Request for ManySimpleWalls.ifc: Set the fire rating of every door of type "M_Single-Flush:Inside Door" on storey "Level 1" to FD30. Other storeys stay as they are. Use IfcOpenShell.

First a look at what the model holds.

```python
import ifcopenshell
import ifcopenshell.util.element

model = ifcopenshell.open("ManySimpleWalls.ifc")
print(model.schema)
storey = next(s for s in model.by_type("IfcBuildingStorey") if s.Name == "Level 1")
doors = [e for e in ifcopenshell.util.element.get_decomposition(storey) if e.is_a("IfcDoor")]
seen = {}
for e in doors:
    element_type = ifcopenshell.util.element.get_type(e)
    key = (element_type.Name if element_type != e and element_type else None, ifcopenshell.util.element.get_pset(e, "Pset_DoorCommon", "FireRating"))
    seen[key] = seen.get(key, 0) + 1
for (name, value), count in sorted(seen.items(), key=str):
    print(count, "x", name, "|", value)
```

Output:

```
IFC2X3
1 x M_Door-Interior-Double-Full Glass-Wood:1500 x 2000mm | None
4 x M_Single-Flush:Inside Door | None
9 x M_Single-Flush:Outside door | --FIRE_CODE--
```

```python
import ifcopenshell
import ifcopenshell.api.pset
import ifcopenshell.util.element

model = ifcopenshell.open("ManySimpleWalls.ifc")

storey = next(s for s in model.by_type("IfcBuildingStorey") if s.Name == "Level 1")
doors = [e for e in ifcopenshell.util.element.get_decomposition(storey) if e.is_a("IfcDoor")]

count = 0
for e in doors:
    element_type = ifcopenshell.util.element.get_type(e)
    if element_type in (None, e) or element_type.Name != "M_Single-Flush:Inside Door":
        continue
    # add_pset returns the element's existing set when there is one.
    pset = ifcopenshell.api.pset.add_pset(model, product=e, name="Pset_DoorCommon")
    ifcopenshell.api.pset.edit_pset(model, pset=pset, properties={"FireRating": "FD30"})
    count += 1

print(count, "doors updated")

model.write("ManySimpleWalls_edited.ifc")
```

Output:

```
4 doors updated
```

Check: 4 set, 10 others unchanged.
